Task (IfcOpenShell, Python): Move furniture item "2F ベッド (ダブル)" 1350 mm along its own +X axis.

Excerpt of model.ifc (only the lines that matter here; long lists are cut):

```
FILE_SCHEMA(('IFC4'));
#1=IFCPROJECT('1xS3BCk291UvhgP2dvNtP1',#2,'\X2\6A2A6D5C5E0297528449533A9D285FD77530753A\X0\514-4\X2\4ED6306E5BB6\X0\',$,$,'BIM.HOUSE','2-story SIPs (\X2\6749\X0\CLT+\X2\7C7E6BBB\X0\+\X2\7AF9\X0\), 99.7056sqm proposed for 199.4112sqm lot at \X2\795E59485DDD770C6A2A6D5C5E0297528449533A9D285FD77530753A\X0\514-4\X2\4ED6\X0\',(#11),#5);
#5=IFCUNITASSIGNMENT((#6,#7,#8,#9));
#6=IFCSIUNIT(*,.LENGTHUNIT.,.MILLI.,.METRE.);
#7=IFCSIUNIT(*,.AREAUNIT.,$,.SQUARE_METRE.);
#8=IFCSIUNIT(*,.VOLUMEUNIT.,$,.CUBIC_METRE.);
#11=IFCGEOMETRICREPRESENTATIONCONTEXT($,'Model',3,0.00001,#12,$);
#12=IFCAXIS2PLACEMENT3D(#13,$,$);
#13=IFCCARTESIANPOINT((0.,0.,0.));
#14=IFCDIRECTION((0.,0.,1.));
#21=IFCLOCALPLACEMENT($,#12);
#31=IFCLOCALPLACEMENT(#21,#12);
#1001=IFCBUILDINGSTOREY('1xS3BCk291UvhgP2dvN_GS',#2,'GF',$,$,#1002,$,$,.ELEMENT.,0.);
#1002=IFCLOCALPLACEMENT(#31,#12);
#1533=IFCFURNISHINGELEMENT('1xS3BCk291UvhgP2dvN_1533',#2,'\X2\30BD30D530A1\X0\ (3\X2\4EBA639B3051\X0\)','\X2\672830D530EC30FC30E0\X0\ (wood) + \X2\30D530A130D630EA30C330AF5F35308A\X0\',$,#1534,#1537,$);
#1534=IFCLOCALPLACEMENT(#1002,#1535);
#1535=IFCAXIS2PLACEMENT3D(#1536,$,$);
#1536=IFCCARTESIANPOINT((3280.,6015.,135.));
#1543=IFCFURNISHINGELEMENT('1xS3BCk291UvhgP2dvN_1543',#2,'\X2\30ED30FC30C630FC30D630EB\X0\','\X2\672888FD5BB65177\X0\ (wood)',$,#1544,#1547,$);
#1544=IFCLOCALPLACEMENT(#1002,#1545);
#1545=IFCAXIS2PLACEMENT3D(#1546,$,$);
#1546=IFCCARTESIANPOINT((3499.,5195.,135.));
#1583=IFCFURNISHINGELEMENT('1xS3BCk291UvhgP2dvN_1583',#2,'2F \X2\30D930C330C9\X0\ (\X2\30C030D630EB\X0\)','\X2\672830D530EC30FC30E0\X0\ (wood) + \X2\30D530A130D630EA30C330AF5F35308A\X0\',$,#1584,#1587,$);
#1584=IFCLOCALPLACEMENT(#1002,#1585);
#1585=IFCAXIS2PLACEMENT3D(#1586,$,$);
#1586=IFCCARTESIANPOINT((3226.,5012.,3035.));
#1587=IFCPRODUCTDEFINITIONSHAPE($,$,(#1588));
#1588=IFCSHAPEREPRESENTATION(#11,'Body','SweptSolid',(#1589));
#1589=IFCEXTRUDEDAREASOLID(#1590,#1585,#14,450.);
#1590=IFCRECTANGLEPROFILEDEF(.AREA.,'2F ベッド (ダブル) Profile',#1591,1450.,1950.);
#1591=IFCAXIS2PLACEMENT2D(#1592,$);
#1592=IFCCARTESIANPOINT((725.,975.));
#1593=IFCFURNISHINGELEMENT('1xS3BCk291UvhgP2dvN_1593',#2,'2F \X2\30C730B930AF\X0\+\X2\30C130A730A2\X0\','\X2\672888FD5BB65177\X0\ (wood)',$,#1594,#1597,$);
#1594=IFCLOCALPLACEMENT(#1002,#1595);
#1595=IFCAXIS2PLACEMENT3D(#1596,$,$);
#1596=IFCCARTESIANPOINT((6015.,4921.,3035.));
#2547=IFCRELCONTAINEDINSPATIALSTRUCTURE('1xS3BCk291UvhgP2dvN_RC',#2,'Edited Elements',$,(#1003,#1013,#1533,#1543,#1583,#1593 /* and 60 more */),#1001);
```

```python
import ifcopenshell
import ifcopenshell.api.geometry
import ifcopenshell.util.placement
import ifcopenshell.util.unit

model = ifcopenshell.open("model.ifc")
unit_scale = ifcopenshell.util.unit.calculate_unit_scale(model)

item = model.by_guid("1xS3BCk291UvhgP2dvN_1583")
matrix = ifcopenshell.util.placement.get_local_placement(item.ObjectPlacement)
matrix[:3, 3] += matrix[:3, 0] * 1.35 / unit_scale
ifcopenshell.api.geometry.edit_object_placement(model, product=item, matrix=matrix, is_si=False)

print(ifcopenshell.util.placement.get_local_placement(item.ObjectPlacement).round(3) + 0.0)

model.write("model_edited.ifc")
```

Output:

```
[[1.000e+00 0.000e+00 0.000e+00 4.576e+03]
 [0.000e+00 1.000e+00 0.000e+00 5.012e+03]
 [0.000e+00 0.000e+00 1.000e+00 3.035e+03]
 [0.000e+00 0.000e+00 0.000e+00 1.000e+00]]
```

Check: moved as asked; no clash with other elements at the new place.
